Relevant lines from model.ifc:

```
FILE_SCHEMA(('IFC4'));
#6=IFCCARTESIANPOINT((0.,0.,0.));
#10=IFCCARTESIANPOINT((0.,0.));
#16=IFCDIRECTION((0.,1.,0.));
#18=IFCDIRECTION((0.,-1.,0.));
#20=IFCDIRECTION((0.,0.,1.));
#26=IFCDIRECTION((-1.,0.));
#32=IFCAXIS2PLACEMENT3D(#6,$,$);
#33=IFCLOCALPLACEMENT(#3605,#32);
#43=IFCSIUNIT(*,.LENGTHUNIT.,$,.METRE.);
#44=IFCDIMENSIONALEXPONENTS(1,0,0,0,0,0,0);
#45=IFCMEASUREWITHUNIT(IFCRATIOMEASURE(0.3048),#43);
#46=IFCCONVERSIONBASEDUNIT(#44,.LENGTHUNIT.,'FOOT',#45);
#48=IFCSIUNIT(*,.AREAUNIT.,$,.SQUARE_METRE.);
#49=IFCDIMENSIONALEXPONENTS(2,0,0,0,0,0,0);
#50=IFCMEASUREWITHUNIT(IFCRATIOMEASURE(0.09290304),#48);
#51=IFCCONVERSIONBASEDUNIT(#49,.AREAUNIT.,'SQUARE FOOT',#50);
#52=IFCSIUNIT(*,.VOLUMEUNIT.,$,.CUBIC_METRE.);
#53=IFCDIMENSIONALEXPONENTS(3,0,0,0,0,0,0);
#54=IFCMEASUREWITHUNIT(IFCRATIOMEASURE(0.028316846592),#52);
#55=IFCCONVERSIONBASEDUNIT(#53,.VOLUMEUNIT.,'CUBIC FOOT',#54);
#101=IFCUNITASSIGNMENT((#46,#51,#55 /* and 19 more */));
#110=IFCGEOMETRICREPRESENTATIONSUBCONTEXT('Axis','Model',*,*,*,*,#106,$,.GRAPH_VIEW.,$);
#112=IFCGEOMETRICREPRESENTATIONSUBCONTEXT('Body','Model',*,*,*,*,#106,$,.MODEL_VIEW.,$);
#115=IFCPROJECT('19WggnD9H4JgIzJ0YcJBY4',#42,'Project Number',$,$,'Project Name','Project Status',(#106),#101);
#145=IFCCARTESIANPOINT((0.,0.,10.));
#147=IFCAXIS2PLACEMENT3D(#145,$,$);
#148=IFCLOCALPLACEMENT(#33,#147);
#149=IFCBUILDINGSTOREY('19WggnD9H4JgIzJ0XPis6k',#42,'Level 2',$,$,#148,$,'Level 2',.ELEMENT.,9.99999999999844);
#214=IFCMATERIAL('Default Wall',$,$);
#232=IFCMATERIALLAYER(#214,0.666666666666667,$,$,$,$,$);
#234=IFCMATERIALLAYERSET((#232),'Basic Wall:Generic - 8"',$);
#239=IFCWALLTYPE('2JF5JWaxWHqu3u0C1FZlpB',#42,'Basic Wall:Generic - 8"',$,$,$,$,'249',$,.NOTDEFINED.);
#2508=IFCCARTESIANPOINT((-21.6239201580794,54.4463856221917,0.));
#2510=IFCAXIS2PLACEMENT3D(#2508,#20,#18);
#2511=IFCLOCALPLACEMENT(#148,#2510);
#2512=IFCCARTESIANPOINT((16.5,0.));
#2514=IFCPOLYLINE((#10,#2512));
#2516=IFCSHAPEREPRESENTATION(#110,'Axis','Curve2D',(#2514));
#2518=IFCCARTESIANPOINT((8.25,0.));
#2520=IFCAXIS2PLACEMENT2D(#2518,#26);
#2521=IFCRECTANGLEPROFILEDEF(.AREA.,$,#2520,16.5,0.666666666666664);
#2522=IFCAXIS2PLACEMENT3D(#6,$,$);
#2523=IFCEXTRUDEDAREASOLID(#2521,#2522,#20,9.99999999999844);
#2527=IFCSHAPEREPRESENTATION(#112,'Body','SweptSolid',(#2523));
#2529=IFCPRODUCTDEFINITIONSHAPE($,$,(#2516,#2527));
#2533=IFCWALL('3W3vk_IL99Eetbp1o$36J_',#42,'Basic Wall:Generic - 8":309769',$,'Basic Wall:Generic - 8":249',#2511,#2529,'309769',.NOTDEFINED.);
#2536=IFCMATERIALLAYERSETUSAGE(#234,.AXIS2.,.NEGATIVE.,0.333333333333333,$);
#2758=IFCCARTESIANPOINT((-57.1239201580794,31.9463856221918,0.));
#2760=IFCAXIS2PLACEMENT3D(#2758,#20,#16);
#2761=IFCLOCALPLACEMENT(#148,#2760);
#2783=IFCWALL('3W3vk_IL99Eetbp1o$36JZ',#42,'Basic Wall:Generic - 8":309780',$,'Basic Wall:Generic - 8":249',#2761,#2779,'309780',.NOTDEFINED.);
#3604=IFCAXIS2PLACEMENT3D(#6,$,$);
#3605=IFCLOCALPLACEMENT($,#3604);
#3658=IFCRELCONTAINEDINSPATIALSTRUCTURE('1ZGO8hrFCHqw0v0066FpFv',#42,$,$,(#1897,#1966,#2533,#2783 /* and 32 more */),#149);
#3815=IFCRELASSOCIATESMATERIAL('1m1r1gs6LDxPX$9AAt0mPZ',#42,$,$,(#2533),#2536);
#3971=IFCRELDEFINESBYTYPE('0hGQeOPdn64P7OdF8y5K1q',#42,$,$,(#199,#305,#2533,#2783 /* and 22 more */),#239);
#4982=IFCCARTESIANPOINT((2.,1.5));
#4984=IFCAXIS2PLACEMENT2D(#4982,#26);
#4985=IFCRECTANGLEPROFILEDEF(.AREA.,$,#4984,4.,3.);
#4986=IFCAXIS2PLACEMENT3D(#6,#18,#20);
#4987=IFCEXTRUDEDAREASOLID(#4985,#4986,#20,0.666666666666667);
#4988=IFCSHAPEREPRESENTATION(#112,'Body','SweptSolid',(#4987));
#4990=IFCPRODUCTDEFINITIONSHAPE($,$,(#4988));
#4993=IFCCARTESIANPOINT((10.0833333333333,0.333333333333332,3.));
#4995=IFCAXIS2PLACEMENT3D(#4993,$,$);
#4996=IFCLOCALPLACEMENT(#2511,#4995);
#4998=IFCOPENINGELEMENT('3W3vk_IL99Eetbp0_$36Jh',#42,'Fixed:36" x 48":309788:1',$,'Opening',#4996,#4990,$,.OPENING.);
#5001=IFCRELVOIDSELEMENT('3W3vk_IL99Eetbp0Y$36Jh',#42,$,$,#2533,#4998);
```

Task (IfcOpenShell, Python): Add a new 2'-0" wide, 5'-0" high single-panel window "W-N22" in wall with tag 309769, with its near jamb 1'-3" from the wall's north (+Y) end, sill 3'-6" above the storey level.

```python
import numpy as np
import ifcopenshell
import ifcopenshell.api.feature
import ifcopenshell.api.geometry
import ifcopenshell.api.root
import ifcopenshell.api.spatial
import ifcopenshell.geom
import ifcopenshell.util.element
import ifcopenshell.util.placement
import ifcopenshell.util.representation
import ifcopenshell.util.shape
import ifcopenshell.util.unit

model = ifcopenshell.open("model.ifc")
unit_scale = ifcopenshell.util.unit.calculate_unit_scale(model)
settings = ifcopenshell.geom.settings()


def volume(element):
    """Net volume in cubic metres, openings subtracted."""
    shape = ifcopenshell.geom.create_shape(settings, element)
    return ifcopenshell.util.shape.get_volume(shape.geometry)


wall = model.by_id(2533)
storey = ifcopenshell.util.element.get_container(wall, ifc_class="IfcBuildingStorey")
context = ifcopenshell.util.representation.get_context(model, "Model", "Body", "MODEL_VIEW")
before = volume(wall)

width, height, from_end, sill = 0.6096, 1.524, 0.381, 1.0668  # metres

# The wall runs along its own X axis, and the end named is its -X end.
wall_shape = ifcopenshell.geom.create_shape(settings, wall)
x, y, z = ifcopenshell.util.shape.get_vertices(wall_shape.geometry).T
start = x.min() + from_end
face, thickness = float(y.min()), float(y.max() - y.min())
wall_matrix = ifcopenshell.util.placement.get_local_placement(wall.ObjectPlacement)
level = ifcopenshell.util.placement.get_local_placement(storey.ObjectPlacement)[2, 3]


def in_wall(x, y):
    """Placement at x, y metres in the wall's axes, at sill height."""
    matrix = wall_matrix.copy()
    matrix[:, 3] = wall_matrix @ np.array([x / unit_scale, y / unit_scale, 0.0, 1.0])
    matrix[2, 3] = level + sill / unit_scale
    return matrix


# Opening: a box that overshoots both wall faces by 50 mm.
opening = ifcopenshell.api.root.create_entity(model, ifc_class="IfcOpeningElement", predefined_type="OPENING")
box = ifcopenshell.api.geometry.add_wall_representation(
    model, context=context, length=width, height=height, thickness=thickness + 0.1
)
ifcopenshell.api.geometry.assign_representation(model, product=opening, representation=box)
ifcopenshell.api.geometry.edit_object_placement(model, product=opening, matrix=in_wall(start, face - 0.05), is_si=False)
ifcopenshell.api.feature.add_feature(model, feature=opening, element=wall)

window = ifcopenshell.api.root.create_entity(model, ifc_class="IfcWindow", name="W-N22", predefined_type="WINDOW")
window.OverallWidth, window.OverallHeight = width / unit_scale, height / unit_scale
window.PartitioningType = "SINGLE_PANEL"
body = ifcopenshell.api.geometry.add_window_representation(
    model,
    context=context,
    overall_width=window.OverallWidth,
    overall_height=window.OverallHeight,
    partition_type="SINGLE_PANEL",
)
ifcopenshell.api.geometry.assign_representation(model, product=window, representation=body)
ifcopenshell.api.spatial.assign_container(model, products=[window], relating_structure=storey)
ifcopenshell.api.feature.add_filling(model, opening=opening, element=window)

# Centre the window in the wall's thickness.
ifcopenshell.api.geometry.edit_object_placement(model, product=window, matrix=in_wall(start, face), is_si=False)
window_shape = ifcopenshell.geom.create_shape(settings, window)
depth = ifcopenshell.util.shape.get_vertices(window_shape.geometry)[:, 1]
offset = face + thickness / 2 - (depth.min() + depth.max()) / 2
ifcopenshell.api.geometry.edit_object_placement(model, product=window, matrix=in_wall(start, offset), is_si=False)

after = volume(wall)

print(f"wall volume {before:.3f} -> {after:.3f} m3")

model.write("model-out.ifc")
```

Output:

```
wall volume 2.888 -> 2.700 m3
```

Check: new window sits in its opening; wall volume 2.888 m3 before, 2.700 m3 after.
